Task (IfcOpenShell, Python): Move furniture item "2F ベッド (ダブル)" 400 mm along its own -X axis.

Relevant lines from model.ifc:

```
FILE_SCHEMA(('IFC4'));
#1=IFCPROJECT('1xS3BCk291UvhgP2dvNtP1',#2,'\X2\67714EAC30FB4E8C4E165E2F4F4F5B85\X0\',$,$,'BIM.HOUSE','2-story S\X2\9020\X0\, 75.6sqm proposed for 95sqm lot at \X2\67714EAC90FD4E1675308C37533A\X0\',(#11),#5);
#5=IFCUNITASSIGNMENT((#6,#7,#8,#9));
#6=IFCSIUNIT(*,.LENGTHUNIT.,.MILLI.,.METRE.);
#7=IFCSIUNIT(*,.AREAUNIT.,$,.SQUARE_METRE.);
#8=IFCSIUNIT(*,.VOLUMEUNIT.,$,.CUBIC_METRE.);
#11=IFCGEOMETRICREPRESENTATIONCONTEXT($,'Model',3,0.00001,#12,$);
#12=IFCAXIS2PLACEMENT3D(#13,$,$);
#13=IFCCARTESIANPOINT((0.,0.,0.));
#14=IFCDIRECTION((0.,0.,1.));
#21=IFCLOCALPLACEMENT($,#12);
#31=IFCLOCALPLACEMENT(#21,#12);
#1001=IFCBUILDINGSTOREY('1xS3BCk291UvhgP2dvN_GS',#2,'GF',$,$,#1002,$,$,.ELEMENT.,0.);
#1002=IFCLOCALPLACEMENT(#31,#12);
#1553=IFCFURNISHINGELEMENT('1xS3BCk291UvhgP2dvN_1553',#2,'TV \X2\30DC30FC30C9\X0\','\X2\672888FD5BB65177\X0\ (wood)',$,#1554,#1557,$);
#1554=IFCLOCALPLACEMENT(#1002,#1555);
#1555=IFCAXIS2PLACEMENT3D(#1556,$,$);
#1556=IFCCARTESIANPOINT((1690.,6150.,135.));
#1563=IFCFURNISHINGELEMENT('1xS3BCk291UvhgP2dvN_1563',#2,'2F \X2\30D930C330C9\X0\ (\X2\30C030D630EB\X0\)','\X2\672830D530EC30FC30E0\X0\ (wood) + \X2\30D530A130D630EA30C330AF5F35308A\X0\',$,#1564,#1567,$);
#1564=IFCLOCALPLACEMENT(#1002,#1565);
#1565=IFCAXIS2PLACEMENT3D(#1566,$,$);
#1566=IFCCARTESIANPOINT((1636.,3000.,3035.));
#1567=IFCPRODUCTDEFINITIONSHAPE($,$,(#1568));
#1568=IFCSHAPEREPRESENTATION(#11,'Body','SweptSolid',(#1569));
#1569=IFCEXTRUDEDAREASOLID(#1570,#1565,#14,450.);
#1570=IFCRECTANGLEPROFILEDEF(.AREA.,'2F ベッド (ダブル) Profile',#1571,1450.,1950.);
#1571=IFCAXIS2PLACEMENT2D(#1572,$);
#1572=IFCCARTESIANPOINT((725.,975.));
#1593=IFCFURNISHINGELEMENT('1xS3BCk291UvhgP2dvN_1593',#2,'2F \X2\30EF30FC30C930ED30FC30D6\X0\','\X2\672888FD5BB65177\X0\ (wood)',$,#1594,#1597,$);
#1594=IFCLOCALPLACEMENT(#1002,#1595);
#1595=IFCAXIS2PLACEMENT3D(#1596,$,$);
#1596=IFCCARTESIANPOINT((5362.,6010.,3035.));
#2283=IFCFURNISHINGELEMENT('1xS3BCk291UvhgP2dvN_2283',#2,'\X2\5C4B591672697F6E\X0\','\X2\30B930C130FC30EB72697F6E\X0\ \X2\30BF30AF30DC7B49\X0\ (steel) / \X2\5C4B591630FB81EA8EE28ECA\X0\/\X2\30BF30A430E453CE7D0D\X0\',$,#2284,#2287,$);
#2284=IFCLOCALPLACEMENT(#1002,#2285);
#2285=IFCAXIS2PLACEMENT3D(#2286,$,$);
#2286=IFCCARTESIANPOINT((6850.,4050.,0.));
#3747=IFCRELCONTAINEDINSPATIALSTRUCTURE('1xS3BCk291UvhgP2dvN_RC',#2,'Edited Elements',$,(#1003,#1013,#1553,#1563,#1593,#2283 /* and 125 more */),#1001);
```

```python
import ifcopenshell
import ifcopenshell.api.geometry
import ifcopenshell.util.placement
import ifcopenshell.util.unit

model = ifcopenshell.open("model.ifc")
unit_scale = ifcopenshell.util.unit.calculate_unit_scale(model)

item = model.by_guid("1xS3BCk291UvhgP2dvN_1563")
matrix = ifcopenshell.util.placement.get_local_placement(item.ObjectPlacement)
matrix[:3, 3] -= matrix[:3, 0] * 0.4 / unit_scale
ifcopenshell.api.geometry.edit_object_placement(model, product=item, matrix=matrix, is_si=False)

print(ifcopenshell.util.placement.get_local_placement(item.ObjectPlacement).round(3) + 0.0)

model.write("model-out.ifc")
```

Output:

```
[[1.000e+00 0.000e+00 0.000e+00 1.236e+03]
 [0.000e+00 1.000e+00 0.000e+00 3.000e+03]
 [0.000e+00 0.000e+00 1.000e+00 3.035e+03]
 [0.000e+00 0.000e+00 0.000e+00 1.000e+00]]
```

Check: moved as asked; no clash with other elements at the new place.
